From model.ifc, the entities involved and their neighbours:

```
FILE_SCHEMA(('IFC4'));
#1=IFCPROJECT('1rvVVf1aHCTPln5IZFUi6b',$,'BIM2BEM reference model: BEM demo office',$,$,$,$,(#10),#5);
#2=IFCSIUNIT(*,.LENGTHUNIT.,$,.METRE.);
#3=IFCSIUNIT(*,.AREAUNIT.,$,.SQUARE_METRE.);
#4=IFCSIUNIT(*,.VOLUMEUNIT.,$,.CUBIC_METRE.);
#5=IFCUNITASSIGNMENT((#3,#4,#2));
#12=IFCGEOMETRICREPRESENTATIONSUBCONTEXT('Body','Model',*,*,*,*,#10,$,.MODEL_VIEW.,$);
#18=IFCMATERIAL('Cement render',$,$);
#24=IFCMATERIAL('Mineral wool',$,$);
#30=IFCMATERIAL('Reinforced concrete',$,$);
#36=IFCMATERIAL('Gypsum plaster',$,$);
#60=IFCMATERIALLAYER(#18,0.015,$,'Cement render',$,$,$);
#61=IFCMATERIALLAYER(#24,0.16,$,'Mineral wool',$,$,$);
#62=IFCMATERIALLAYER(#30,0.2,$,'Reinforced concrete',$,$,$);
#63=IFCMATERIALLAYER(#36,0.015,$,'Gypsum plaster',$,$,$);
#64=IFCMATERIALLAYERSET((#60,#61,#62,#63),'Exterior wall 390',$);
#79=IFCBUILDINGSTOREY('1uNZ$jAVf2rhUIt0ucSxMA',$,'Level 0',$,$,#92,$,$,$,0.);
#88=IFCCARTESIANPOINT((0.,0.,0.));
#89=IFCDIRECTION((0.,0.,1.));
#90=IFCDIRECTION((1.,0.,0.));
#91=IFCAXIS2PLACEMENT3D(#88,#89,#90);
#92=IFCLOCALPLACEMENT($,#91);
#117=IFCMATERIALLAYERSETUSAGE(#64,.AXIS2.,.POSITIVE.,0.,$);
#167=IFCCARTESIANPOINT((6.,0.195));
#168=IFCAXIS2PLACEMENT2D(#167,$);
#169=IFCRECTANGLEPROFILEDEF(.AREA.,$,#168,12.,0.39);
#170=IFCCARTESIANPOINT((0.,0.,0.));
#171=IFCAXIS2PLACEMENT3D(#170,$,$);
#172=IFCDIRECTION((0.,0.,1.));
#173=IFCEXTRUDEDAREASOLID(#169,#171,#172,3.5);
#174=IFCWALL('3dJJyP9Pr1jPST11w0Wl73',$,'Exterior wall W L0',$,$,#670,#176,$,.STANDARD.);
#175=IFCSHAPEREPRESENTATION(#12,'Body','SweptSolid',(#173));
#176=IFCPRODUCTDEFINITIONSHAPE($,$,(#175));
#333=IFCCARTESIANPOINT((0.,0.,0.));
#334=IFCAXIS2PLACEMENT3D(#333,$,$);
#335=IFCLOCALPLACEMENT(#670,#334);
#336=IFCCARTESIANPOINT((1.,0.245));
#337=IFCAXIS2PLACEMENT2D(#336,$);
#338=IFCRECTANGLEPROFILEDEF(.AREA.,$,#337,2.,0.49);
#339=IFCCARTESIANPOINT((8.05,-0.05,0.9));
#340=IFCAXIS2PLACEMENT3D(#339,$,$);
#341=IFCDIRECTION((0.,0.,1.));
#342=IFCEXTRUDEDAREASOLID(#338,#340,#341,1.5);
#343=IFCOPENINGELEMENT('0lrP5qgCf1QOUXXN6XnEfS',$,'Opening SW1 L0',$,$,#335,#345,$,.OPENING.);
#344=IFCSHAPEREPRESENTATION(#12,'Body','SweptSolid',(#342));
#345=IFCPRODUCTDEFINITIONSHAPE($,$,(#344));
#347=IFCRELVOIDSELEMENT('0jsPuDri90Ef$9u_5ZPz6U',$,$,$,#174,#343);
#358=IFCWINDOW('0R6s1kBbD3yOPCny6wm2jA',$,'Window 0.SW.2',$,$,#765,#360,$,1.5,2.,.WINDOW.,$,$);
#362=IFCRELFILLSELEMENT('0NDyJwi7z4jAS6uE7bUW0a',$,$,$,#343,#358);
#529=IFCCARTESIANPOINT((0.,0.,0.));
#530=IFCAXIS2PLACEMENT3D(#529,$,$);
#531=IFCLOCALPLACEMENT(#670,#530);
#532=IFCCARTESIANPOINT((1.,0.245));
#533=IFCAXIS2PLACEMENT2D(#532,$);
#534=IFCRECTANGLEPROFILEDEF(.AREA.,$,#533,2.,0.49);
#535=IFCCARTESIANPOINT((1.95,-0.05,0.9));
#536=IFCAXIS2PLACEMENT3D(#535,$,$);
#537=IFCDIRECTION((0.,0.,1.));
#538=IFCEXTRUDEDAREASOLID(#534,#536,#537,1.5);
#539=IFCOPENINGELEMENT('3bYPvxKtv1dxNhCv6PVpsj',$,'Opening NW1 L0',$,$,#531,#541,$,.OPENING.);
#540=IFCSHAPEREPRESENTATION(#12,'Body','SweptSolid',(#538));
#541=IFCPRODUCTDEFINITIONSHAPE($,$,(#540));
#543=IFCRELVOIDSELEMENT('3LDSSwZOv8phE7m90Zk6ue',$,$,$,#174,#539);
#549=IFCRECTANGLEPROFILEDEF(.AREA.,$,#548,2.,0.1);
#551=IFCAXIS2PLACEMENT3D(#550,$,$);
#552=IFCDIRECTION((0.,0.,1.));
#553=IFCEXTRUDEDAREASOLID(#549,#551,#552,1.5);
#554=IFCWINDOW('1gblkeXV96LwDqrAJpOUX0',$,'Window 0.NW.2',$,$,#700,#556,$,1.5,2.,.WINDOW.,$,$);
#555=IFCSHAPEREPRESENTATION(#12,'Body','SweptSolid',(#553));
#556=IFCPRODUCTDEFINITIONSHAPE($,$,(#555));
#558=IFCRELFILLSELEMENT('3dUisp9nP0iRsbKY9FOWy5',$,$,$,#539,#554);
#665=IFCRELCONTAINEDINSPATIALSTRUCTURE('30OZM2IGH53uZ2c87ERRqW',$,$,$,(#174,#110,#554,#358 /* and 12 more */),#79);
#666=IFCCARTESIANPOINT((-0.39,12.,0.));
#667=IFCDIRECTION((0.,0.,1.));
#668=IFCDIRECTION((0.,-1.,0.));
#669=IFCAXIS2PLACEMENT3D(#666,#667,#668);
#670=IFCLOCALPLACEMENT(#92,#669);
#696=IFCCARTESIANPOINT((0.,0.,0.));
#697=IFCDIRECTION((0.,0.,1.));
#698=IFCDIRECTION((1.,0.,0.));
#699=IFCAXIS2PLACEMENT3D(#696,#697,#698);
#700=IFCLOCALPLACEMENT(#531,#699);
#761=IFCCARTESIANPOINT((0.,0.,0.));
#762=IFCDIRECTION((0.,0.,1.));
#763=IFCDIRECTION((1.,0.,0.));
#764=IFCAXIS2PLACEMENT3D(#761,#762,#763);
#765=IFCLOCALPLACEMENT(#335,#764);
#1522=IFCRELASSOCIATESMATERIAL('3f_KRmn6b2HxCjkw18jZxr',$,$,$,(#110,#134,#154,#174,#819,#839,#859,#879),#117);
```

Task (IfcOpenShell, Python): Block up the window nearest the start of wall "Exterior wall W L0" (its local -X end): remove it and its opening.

```python
import ifcopenshell
import ifcopenshell.api.feature
import ifcopenshell.api.root
import ifcopenshell.geom
import ifcopenshell.util.shape

model = ifcopenshell.open("model.ifc")
settings = ifcopenshell.geom.settings()


def volume(element):
    """Net volume in cubic metres, openings subtracted."""
    shape = ifcopenshell.geom.create_shape(settings, element)
    return ifcopenshell.util.shape.get_volume(shape.geometry)


window = model.by_guid("1gblkeXV96LwDqrAJpOUX0")
opening = window.FillsVoids[0].RelatingOpeningElement
wall = opening.VoidsElements[0].RelatingBuildingElement
before = volume(wall)

ifcopenshell.api.root.remove_product(model, product=window)
ifcopenshell.api.feature.remove_feature(model, feature=opening)

after = volume(wall)

print(f"wall volume {before:.3f} -> {after:.3f} m3")

model.write("model_rev.ifc")
```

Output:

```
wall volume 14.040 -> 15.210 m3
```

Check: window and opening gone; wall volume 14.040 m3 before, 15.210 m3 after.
